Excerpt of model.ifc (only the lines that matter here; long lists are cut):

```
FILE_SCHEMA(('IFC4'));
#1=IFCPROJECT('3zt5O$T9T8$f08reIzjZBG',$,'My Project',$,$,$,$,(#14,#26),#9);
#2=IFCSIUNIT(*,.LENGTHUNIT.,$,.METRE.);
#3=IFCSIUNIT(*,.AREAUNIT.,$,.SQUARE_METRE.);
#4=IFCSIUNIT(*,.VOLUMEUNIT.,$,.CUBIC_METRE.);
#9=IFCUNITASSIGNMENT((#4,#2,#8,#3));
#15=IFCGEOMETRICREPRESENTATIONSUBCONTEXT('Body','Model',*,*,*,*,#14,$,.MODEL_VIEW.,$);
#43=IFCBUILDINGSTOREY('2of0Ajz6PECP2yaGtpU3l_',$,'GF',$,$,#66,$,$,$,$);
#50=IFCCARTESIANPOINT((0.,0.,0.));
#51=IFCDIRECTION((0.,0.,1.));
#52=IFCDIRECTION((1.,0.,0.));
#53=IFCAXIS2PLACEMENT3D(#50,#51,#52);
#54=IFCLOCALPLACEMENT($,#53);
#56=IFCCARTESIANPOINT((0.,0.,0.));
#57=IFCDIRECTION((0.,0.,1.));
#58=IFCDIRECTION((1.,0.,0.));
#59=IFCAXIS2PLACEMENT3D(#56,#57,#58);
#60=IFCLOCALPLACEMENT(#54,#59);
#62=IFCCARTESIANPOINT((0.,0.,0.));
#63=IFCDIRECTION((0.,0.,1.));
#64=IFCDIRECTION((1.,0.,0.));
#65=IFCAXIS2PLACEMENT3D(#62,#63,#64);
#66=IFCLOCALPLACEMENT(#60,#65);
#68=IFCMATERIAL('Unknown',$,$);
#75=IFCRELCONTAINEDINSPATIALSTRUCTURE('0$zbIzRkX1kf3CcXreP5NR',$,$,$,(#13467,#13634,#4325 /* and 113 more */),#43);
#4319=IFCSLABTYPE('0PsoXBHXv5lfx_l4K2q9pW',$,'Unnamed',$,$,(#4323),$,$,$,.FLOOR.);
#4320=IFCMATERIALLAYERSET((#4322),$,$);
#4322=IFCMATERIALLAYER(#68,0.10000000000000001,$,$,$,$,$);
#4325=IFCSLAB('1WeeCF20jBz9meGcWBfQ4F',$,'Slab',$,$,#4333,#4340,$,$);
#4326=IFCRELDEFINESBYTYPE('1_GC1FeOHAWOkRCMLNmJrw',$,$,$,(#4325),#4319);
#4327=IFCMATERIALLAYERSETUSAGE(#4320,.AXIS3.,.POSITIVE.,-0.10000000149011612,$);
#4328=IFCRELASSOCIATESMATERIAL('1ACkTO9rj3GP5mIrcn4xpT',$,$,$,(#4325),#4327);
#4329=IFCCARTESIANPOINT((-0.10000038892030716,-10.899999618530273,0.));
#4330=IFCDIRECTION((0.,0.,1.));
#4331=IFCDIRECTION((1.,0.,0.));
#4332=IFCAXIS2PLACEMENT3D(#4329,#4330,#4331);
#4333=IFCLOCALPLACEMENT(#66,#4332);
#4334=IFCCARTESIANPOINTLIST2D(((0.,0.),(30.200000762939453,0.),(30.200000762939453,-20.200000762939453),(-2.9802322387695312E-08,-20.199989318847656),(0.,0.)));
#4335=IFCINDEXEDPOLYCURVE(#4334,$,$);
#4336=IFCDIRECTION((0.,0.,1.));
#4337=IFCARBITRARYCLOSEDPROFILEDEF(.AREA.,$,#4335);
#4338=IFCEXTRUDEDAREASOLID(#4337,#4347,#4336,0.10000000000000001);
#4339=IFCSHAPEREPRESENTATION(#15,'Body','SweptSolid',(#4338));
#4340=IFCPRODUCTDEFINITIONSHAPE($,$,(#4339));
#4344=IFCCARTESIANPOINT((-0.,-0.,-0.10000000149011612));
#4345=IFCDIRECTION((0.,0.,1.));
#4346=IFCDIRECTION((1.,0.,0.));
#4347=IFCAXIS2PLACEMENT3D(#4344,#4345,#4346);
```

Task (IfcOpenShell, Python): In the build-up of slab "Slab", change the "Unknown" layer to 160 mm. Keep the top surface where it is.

```python
import ifcopenshell
import ifcopenshell.util.element
import ifcopenshell.util.representation
import ifcopenshell.util.unit

model = ifcopenshell.open("model.ifc")
unit_scale = ifcopenshell.util.unit.calculate_unit_scale(model)

layer_set = model.by_id(4320)
layer = next(l for l in layer_set.MaterialLayers if l.Material and l.Material.Name == "Unknown")
change = 0.16 / unit_scale - layer.LayerThickness
layer.LayerThickness += change

# Geometry does not follow the layer set by itself.
slabs = [e for e in ifcopenshell.util.element.get_elements_by_material(model, layer_set) if e.is_a("IfcSlab")]
for slab in sorted(slabs, key=lambda e: e.id()):
    body = ifcopenshell.util.representation.get_representation(slab, "Model", "Body")
    solid = body.Items[0]
    old_depth = solid.Depth
    solid.Depth += change
    # Extruded upwards: lower the start of the extrusion so the top stays.
    x, y, z = solid.Position.Location.Coordinates
    solid.Position.Location = model.createIfcCartesianPoint((x, y, z - change))
    print(slab.id(), f"{old_depth:g} -> {solid.Depth:g}")

# The layers are counted up from the underside, which has moved.
for usage in {ifcopenshell.util.element.get_material(slab) for slab in slabs}:
    usage.OffsetFromReferenceLine -= change

model.write("model_rev.ifc")
```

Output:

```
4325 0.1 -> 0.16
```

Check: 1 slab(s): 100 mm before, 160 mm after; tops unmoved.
